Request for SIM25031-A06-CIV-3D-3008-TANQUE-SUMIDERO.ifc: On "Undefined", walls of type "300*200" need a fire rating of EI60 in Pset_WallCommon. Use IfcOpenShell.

First a look at what the model holds.

```python
import ifcopenshell
import ifcopenshell.util.element

model = ifcopenshell.open("SIM25031-A06-CIV-3D-3008-TANQUE-SUMIDERO.ifc")
print(model.schema)
storey = next(s for s in model.by_type("IfcBuildingStorey") if s.Name == "Undefined")
walls = [e for e in ifcopenshell.util.element.get_decomposition(storey) if e.is_a("IfcWall")]
seen = {}
for e in walls:
    element_type = ifcopenshell.util.element.get_type(e)
    key = (element_type.Name if element_type != e and element_type else None, ifcopenshell.util.element.get_pset(e, "Pset_WallCommon", "FireRating"))
    seen[key] = seen.get(key, 0) + 1
for (name, value), count in sorted(seen.items(), key=str):
    print(count, "x", name, "|", value)
```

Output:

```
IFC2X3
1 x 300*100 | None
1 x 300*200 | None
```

```python
import ifcopenshell
import ifcopenshell.api.pset
import ifcopenshell.util.element

model = ifcopenshell.open("SIM25031-A06-CIV-3D-3008-TANQUE-SUMIDERO.ifc")

storey = next(s for s in model.by_type("IfcBuildingStorey") if s.Name == "Undefined")
walls = [e for e in ifcopenshell.util.element.get_decomposition(storey) if e.is_a("IfcWall")]

count = 0
for e in walls:
    element_type = ifcopenshell.util.element.get_type(e)
    if element_type in (None, e) or element_type.Name != "300*200":
        continue
    # add_pset returns the element's existing set when there is one.
    pset = ifcopenshell.api.pset.add_pset(model, product=e, name="Pset_WallCommon")
    ifcopenshell.api.pset.edit_pset(model, pset=pset, properties={"FireRating": "EI60"})
    count += 1

print(count, "walls updated")

model.write("SIM25031-A06-CIV-3D-3008-TANQUE-SUMIDERO-out.ifc")
```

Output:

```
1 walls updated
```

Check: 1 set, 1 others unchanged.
